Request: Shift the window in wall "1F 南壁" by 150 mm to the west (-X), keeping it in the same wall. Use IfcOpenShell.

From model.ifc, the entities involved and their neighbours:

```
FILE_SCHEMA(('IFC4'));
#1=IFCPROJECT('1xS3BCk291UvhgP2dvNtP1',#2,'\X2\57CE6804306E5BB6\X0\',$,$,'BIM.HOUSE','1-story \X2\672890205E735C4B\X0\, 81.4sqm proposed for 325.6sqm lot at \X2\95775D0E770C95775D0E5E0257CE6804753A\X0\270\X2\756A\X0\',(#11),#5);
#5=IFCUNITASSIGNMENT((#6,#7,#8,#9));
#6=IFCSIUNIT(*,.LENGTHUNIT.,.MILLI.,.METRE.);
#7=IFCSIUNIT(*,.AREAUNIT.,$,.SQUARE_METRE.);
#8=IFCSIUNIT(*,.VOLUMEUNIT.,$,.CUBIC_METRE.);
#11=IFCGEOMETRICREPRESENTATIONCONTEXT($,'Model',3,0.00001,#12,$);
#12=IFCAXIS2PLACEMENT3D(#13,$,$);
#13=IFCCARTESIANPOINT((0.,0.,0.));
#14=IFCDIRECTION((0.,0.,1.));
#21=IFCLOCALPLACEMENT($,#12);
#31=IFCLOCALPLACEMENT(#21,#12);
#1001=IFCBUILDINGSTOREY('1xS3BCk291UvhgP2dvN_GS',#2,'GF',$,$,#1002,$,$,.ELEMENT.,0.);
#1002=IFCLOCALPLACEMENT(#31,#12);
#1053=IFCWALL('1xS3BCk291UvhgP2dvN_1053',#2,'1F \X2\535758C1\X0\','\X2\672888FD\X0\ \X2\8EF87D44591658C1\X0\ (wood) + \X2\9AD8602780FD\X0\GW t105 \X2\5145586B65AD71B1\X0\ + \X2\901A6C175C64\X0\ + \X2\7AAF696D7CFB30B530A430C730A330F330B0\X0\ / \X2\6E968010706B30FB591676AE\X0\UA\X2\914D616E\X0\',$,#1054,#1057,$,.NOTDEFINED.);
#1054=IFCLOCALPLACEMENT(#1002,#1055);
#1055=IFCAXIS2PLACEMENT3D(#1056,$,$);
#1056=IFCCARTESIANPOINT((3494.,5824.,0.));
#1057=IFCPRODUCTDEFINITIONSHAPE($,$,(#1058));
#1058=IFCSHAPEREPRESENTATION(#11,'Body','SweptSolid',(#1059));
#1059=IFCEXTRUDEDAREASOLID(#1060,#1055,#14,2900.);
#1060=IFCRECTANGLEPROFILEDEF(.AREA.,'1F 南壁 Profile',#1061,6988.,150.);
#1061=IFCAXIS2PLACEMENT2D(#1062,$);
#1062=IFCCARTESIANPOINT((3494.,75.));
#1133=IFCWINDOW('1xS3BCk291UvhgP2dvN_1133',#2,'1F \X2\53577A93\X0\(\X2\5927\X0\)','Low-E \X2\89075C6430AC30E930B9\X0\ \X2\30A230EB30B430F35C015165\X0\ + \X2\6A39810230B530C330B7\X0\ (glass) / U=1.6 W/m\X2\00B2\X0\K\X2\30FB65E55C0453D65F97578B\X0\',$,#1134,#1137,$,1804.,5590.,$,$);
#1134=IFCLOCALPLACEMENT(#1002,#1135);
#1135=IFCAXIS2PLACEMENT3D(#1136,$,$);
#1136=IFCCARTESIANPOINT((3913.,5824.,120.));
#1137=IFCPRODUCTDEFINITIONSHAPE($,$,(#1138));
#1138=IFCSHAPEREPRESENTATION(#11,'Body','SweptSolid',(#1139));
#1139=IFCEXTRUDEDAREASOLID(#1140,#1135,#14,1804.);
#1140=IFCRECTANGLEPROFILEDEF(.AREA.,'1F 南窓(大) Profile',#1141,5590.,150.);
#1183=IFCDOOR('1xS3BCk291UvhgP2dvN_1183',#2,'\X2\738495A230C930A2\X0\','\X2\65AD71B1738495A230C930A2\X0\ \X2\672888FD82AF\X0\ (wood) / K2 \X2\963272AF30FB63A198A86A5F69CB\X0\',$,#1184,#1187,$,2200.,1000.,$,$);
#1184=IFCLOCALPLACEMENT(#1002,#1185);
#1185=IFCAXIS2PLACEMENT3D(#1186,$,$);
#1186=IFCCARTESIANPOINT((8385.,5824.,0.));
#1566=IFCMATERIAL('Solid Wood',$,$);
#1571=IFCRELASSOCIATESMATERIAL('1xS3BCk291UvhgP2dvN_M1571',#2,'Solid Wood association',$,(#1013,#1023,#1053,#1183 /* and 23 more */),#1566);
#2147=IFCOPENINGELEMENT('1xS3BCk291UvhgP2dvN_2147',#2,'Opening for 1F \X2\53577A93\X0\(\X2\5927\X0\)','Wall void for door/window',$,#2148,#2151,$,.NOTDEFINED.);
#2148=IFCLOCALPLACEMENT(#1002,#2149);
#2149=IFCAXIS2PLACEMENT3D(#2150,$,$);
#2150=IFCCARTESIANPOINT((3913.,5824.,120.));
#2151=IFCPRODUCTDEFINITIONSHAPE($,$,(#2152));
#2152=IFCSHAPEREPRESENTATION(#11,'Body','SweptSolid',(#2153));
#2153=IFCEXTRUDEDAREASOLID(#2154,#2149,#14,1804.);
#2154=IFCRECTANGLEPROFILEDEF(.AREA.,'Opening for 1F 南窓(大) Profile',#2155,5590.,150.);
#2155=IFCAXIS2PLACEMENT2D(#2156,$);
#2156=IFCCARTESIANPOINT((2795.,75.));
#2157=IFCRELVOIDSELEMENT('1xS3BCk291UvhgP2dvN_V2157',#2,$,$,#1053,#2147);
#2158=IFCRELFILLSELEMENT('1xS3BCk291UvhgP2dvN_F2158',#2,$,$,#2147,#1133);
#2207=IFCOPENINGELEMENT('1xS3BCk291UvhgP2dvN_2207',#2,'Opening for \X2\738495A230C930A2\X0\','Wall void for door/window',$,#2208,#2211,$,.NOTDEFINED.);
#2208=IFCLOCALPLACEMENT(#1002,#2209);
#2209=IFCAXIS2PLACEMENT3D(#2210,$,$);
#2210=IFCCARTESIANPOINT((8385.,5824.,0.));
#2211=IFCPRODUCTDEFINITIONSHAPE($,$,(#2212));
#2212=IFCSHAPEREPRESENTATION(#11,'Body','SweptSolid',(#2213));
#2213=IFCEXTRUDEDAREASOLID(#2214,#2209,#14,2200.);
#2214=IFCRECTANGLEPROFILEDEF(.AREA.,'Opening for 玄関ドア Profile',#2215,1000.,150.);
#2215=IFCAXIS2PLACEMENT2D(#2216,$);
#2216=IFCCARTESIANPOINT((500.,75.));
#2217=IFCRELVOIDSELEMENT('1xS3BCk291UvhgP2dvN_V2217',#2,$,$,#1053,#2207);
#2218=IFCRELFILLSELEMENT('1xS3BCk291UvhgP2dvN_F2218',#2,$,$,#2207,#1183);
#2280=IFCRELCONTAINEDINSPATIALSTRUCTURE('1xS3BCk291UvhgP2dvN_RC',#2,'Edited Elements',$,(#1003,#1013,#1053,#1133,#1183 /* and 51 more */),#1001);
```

```python
import ifcopenshell
import ifcopenshell.api.geometry
import ifcopenshell.util.placement
import ifcopenshell.util.unit

model = ifcopenshell.open("model.ifc")
unit_scale = ifcopenshell.util.unit.calculate_unit_scale(model)

window = model.by_guid("1xS3BCk291UvhgP2dvN_1133")
opening = window.FillsVoids[0].RelatingOpeningElement
wall = opening.VoidsElements[0].RelatingBuildingElement

wall_matrix = ifcopenshell.util.placement.get_local_placement(wall.ObjectPlacement)
shift = wall_matrix[:3, 0] * -0.15 / unit_scale
before = ifcopenshell.util.placement.get_local_placement(window.ObjectPlacement)[:3, 3].copy()

# The window is not placed relative to its opening, so move both.
for product in (opening, window):
    matrix = ifcopenshell.util.placement.get_local_placement(product.ObjectPlacement)
    matrix[:3, 3] += shift
    ifcopenshell.api.geometry.edit_object_placement(model, product=product, matrix=matrix, is_si=False)

after = ifcopenshell.util.placement.get_local_placement(window.ObjectPlacement)[:3, 3]
print("window moved by", (after - before).round(3) + 0.0)

model.write("model_rev.ifc")
```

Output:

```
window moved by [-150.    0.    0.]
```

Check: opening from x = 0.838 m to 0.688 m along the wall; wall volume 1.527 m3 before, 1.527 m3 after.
